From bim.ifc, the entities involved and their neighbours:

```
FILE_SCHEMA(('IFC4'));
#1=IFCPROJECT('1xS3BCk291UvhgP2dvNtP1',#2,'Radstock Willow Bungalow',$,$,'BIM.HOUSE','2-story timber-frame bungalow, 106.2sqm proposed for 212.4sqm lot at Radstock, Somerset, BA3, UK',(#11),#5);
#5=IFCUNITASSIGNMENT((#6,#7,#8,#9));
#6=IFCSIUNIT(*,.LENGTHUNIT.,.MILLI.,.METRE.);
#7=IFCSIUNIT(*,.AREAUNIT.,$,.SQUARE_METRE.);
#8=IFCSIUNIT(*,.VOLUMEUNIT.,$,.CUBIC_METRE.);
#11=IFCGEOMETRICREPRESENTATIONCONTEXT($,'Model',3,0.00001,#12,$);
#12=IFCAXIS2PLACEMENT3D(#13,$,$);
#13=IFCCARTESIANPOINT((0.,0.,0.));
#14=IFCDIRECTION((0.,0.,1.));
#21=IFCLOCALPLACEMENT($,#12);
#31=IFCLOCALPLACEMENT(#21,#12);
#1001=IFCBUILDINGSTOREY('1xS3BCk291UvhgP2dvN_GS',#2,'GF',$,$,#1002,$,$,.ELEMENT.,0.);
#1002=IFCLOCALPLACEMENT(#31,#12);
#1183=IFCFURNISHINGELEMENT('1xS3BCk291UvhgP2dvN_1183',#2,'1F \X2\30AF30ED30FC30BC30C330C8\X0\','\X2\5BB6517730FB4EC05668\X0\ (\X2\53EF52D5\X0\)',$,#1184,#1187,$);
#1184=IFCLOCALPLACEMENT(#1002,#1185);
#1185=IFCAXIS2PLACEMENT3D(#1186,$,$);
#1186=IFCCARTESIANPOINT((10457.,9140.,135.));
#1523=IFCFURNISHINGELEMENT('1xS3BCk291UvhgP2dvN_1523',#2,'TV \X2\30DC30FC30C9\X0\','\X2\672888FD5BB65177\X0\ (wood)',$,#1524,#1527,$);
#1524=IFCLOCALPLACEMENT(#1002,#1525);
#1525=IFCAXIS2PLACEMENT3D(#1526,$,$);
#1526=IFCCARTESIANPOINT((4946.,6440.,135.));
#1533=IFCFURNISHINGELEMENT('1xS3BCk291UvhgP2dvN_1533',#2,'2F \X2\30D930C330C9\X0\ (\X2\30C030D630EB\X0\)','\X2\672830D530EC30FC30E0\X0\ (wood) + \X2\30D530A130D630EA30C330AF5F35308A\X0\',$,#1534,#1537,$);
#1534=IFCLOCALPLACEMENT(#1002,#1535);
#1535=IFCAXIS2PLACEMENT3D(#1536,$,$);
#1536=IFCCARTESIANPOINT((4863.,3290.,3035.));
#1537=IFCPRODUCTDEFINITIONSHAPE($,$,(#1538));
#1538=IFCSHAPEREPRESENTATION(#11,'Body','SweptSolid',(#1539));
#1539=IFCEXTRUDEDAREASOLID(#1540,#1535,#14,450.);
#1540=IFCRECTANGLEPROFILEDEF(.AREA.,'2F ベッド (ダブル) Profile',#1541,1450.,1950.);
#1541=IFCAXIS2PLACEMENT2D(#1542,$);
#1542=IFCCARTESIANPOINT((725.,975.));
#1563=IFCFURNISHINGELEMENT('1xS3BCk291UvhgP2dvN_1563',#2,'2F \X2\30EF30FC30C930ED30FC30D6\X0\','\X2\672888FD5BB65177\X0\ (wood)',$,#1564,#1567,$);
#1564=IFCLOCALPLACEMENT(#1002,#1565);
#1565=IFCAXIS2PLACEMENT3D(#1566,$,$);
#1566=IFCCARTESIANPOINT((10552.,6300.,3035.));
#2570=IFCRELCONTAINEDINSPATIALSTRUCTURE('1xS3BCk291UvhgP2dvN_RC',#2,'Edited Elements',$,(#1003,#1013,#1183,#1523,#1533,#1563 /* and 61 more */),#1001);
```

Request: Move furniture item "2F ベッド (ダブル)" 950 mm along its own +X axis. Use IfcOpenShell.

```python
import ifcopenshell
import ifcopenshell.api.geometry
import ifcopenshell.util.placement

model = ifcopenshell.open("bim.ifc")

item = model.by_id(1533)
matrix = ifcopenshell.util.placement.get_local_placement(item.ObjectPlacement)
matrix[:3, 3] += matrix[:3, 0] * 950.0
ifcopenshell.api.geometry.edit_object_placement(model, product=item, matrix=matrix, is_si=False)

print(ifcopenshell.util.placement.get_local_placement(item.ObjectPlacement).round(3) + 0.0)

model.write("bim_edited.ifc")
```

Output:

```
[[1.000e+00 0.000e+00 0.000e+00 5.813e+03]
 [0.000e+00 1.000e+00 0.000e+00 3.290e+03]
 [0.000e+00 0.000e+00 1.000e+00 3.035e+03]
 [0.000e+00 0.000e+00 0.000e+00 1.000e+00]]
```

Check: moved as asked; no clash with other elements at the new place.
